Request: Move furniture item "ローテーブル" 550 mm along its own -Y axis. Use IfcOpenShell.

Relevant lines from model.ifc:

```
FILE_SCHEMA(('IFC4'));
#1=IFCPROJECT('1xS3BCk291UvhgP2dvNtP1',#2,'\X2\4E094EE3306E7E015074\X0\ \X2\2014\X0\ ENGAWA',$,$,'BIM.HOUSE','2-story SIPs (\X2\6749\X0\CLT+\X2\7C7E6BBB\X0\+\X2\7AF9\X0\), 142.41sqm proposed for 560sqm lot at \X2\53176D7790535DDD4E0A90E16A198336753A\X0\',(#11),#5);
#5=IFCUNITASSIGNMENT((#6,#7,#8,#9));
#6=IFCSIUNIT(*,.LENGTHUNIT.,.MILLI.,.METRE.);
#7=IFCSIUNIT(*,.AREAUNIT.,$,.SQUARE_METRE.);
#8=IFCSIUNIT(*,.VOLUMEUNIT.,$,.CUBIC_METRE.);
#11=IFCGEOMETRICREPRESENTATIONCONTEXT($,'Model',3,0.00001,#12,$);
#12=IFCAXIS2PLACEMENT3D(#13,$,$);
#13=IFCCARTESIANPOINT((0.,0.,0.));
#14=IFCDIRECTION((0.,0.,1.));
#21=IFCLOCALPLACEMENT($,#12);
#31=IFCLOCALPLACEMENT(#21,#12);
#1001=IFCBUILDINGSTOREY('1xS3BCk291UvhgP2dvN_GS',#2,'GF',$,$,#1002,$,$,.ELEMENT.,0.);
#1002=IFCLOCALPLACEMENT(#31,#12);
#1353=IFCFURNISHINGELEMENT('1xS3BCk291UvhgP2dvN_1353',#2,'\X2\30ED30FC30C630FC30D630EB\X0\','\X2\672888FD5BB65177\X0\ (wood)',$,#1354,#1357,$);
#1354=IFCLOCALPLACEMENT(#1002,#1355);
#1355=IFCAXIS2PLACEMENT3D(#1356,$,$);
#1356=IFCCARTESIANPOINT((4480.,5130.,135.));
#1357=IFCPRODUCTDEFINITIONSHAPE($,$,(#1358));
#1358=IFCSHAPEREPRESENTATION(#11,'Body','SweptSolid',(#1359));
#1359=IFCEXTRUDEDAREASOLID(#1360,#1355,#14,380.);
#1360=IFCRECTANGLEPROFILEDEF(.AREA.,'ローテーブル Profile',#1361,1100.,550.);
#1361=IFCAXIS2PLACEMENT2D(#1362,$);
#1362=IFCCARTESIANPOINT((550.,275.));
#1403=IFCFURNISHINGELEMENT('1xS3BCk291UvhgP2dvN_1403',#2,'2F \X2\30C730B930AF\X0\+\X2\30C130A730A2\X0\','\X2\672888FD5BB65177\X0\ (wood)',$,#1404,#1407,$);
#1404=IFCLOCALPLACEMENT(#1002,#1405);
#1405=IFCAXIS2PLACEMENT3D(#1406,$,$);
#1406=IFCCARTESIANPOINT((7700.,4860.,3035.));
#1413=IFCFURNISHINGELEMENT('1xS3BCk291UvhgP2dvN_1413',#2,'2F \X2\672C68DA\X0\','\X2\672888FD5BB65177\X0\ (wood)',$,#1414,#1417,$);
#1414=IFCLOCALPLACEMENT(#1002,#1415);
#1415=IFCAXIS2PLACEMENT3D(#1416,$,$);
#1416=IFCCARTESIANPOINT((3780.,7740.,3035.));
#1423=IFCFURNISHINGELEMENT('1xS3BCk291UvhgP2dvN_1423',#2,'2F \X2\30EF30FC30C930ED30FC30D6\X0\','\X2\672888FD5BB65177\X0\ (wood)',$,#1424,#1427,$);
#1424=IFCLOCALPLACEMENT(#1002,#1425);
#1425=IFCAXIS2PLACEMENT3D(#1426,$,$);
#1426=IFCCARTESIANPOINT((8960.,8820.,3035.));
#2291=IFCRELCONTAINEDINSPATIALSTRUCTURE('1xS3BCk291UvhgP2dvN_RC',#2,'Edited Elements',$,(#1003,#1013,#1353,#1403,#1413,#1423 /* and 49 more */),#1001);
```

```python
import ifcopenshell
import ifcopenshell.api.geometry
import ifcopenshell.util.placement
import ifcopenshell.util.unit

model = ifcopenshell.open("model.ifc")
unit_scale = ifcopenshell.util.unit.calculate_unit_scale(model)

item = model.by_guid("1xS3BCk291UvhgP2dvN_1353")
matrix = ifcopenshell.util.placement.get_local_placement(item.ObjectPlacement)
matrix[:3, 3] -= matrix[:3, 1] * 0.55 / unit_scale
ifcopenshell.api.geometry.edit_object_placement(model, product=item, matrix=matrix, is_si=False)

print(ifcopenshell.util.placement.get_local_placement(item.ObjectPlacement).round(3) + 0.0)

model.write("model_v2.ifc")
```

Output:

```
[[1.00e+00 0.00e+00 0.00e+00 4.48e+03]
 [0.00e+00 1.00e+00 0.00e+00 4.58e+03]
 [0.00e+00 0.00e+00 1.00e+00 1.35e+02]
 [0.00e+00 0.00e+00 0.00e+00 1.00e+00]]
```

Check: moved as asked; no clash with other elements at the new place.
